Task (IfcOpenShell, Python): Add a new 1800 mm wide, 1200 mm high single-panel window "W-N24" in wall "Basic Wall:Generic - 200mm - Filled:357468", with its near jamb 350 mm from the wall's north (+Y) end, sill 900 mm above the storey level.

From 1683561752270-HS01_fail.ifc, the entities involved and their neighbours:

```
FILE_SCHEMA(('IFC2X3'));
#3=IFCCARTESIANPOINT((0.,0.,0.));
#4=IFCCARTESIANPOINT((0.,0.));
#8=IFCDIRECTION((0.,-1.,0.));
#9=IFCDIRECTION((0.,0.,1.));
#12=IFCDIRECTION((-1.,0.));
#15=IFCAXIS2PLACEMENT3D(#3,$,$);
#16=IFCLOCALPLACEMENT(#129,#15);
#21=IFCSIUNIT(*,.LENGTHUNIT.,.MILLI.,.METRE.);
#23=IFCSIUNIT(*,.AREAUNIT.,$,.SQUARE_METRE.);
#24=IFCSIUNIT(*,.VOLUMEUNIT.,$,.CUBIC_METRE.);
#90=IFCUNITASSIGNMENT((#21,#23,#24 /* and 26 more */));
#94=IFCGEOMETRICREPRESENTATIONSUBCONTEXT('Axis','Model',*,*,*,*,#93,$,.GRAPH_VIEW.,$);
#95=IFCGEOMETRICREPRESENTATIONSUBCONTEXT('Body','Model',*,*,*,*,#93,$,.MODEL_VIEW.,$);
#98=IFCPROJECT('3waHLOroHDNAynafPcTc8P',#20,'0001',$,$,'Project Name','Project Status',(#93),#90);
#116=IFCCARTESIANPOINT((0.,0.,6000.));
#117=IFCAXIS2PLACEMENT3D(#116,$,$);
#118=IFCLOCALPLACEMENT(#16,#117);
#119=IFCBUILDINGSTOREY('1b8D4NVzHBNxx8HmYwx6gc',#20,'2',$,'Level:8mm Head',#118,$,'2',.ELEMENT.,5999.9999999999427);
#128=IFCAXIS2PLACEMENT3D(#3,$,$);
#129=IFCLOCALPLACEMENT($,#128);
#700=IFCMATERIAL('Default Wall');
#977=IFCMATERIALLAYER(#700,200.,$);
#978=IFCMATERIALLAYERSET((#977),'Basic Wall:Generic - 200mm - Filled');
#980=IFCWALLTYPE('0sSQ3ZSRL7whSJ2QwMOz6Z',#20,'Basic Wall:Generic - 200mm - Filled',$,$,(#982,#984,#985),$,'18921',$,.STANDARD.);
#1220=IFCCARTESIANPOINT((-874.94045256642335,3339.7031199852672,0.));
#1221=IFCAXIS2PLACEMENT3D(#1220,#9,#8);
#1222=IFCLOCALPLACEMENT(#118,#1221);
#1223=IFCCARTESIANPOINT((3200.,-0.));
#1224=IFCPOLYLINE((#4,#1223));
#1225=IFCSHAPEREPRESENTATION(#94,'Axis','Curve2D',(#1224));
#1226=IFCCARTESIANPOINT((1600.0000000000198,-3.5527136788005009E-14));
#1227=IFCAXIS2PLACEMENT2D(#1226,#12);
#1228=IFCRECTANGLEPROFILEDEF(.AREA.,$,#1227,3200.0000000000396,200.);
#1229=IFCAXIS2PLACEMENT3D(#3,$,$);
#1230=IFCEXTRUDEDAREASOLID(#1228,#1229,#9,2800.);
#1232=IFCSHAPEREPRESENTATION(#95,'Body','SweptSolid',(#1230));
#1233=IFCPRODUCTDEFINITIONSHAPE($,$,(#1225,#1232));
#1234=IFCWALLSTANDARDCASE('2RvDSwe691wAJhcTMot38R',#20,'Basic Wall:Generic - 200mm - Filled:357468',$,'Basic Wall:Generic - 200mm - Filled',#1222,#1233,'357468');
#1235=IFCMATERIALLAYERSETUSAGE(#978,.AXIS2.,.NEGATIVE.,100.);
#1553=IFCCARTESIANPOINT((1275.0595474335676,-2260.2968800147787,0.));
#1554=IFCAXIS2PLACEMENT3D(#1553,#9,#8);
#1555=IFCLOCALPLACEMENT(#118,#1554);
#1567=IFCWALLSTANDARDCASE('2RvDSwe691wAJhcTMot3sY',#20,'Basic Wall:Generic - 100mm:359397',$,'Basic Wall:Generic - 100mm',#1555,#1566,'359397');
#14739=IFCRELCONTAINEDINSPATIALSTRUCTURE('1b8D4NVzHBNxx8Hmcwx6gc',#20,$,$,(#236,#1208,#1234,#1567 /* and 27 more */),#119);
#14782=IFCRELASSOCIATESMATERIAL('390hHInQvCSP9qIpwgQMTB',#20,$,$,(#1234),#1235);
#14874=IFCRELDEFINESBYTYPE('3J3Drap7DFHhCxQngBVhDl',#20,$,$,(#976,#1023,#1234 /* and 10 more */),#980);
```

```python
import numpy as np
import ifcopenshell
import ifcopenshell.api.feature
import ifcopenshell.api.geometry
import ifcopenshell.api.root
import ifcopenshell.api.spatial
import ifcopenshell.api.type
import ifcopenshell.geom
import ifcopenshell.util.element
import ifcopenshell.util.placement
import ifcopenshell.util.representation
import ifcopenshell.util.shape
import ifcopenshell.util.unit

model = ifcopenshell.open("1683561752270-HS01_fail.ifc")
unit_scale = ifcopenshell.util.unit.calculate_unit_scale(model)
settings = ifcopenshell.geom.settings()


def volume(element):
    """Net volume in cubic metres, openings subtracted."""
    shape = ifcopenshell.geom.create_shape(settings, element)
    return ifcopenshell.util.shape.get_volume(shape.geometry)


wall = model.by_id(1234)
storey = ifcopenshell.util.element.get_container(wall, ifc_class="IfcBuildingStorey")
context = ifcopenshell.util.representation.get_context(model, "Model", "Body", "MODEL_VIEW")
before = volume(wall)

width, height, from_end, sill = 1.8, 1.2, 0.35, 0.9  # metres

# The wall runs along its own X axis, and the end named is its -X end.
wall_shape = ifcopenshell.geom.create_shape(settings, wall)
x, y, z = ifcopenshell.util.shape.get_vertices(wall_shape.geometry).T
start = x.min() + from_end
face, thickness = float(y.min()), float(y.max() - y.min())
wall_matrix = ifcopenshell.util.placement.get_local_placement(wall.ObjectPlacement)
level = ifcopenshell.util.placement.get_local_placement(storey.ObjectPlacement)[2, 3]


def in_wall(x, y):
    """Placement at x, y metres in the wall's axes, at sill height."""
    matrix = wall_matrix.copy()
    matrix[:, 3] = wall_matrix @ np.array([x / unit_scale, y / unit_scale, 0.0, 1.0])
    matrix[2, 3] = level + sill / unit_scale
    return matrix


# Opening: a box that overshoots both wall faces by 50 mm.
opening = ifcopenshell.api.root.create_entity(model, ifc_class="IfcOpeningElement")
box = ifcopenshell.api.geometry.add_wall_representation(
    model, context=context, length=width, height=height, thickness=thickness + 0.1
)
ifcopenshell.api.geometry.assign_representation(model, product=opening, representation=box)
ifcopenshell.api.geometry.edit_object_placement(model, product=opening, matrix=in_wall(start, face - 0.05), is_si=False)
ifcopenshell.api.feature.add_feature(model, feature=opening, element=wall)

window = ifcopenshell.api.root.create_entity(model, ifc_class="IfcWindow", name="W-N24")
window.OverallWidth, window.OverallHeight = width / unit_scale, height / unit_scale
body = ifcopenshell.api.geometry.add_window_representation(
    model,
    context=context,
    overall_width=window.OverallWidth,
    overall_height=window.OverallHeight,
    partition_type="SINGLE_PANEL",
)
ifcopenshell.api.geometry.assign_representation(model, product=window, representation=body)
ifcopenshell.api.spatial.assign_container(model, products=[window], relating_structure=storey)
fills = ifcopenshell.api.feature.add_filling(model, opening=opening, element=window)
fills.OwnerHistory = window.OwnerHistory  # required in IFC2X3

# IFC2X3 keeps the operation on the window style.
style = ifcopenshell.api.root.create_entity(model, ifc_class="IfcWindowStyle", name="W-N24")
style.OperationType, style.ConstructionType = "SINGLE_PANEL", "NOTDEFINED"
style.ParameterTakesPrecedence = style.Sizeable = False
ifcopenshell.api.type.assign_type(model, related_objects=[window], relating_type=style)

# Centre the window in the wall's thickness.
ifcopenshell.api.geometry.edit_object_placement(model, product=window, matrix=in_wall(start, face), is_si=False)
window_shape = ifcopenshell.geom.create_shape(settings, window)
depth = ifcopenshell.util.shape.get_vertices(window_shape.geometry)[:, 1]
offset = face + thickness / 2 - (depth.min() + depth.max()) / 2
ifcopenshell.api.geometry.edit_object_placement(model, product=window, matrix=in_wall(start, offset), is_si=False)

after = volume(wall)

print(f"wall volume {before:.3f} -> {after:.3f} m3")

model.write("1683561752270-HS01_fail_edited.ifc")
```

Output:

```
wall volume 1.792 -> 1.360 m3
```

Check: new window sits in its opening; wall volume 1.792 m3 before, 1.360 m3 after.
